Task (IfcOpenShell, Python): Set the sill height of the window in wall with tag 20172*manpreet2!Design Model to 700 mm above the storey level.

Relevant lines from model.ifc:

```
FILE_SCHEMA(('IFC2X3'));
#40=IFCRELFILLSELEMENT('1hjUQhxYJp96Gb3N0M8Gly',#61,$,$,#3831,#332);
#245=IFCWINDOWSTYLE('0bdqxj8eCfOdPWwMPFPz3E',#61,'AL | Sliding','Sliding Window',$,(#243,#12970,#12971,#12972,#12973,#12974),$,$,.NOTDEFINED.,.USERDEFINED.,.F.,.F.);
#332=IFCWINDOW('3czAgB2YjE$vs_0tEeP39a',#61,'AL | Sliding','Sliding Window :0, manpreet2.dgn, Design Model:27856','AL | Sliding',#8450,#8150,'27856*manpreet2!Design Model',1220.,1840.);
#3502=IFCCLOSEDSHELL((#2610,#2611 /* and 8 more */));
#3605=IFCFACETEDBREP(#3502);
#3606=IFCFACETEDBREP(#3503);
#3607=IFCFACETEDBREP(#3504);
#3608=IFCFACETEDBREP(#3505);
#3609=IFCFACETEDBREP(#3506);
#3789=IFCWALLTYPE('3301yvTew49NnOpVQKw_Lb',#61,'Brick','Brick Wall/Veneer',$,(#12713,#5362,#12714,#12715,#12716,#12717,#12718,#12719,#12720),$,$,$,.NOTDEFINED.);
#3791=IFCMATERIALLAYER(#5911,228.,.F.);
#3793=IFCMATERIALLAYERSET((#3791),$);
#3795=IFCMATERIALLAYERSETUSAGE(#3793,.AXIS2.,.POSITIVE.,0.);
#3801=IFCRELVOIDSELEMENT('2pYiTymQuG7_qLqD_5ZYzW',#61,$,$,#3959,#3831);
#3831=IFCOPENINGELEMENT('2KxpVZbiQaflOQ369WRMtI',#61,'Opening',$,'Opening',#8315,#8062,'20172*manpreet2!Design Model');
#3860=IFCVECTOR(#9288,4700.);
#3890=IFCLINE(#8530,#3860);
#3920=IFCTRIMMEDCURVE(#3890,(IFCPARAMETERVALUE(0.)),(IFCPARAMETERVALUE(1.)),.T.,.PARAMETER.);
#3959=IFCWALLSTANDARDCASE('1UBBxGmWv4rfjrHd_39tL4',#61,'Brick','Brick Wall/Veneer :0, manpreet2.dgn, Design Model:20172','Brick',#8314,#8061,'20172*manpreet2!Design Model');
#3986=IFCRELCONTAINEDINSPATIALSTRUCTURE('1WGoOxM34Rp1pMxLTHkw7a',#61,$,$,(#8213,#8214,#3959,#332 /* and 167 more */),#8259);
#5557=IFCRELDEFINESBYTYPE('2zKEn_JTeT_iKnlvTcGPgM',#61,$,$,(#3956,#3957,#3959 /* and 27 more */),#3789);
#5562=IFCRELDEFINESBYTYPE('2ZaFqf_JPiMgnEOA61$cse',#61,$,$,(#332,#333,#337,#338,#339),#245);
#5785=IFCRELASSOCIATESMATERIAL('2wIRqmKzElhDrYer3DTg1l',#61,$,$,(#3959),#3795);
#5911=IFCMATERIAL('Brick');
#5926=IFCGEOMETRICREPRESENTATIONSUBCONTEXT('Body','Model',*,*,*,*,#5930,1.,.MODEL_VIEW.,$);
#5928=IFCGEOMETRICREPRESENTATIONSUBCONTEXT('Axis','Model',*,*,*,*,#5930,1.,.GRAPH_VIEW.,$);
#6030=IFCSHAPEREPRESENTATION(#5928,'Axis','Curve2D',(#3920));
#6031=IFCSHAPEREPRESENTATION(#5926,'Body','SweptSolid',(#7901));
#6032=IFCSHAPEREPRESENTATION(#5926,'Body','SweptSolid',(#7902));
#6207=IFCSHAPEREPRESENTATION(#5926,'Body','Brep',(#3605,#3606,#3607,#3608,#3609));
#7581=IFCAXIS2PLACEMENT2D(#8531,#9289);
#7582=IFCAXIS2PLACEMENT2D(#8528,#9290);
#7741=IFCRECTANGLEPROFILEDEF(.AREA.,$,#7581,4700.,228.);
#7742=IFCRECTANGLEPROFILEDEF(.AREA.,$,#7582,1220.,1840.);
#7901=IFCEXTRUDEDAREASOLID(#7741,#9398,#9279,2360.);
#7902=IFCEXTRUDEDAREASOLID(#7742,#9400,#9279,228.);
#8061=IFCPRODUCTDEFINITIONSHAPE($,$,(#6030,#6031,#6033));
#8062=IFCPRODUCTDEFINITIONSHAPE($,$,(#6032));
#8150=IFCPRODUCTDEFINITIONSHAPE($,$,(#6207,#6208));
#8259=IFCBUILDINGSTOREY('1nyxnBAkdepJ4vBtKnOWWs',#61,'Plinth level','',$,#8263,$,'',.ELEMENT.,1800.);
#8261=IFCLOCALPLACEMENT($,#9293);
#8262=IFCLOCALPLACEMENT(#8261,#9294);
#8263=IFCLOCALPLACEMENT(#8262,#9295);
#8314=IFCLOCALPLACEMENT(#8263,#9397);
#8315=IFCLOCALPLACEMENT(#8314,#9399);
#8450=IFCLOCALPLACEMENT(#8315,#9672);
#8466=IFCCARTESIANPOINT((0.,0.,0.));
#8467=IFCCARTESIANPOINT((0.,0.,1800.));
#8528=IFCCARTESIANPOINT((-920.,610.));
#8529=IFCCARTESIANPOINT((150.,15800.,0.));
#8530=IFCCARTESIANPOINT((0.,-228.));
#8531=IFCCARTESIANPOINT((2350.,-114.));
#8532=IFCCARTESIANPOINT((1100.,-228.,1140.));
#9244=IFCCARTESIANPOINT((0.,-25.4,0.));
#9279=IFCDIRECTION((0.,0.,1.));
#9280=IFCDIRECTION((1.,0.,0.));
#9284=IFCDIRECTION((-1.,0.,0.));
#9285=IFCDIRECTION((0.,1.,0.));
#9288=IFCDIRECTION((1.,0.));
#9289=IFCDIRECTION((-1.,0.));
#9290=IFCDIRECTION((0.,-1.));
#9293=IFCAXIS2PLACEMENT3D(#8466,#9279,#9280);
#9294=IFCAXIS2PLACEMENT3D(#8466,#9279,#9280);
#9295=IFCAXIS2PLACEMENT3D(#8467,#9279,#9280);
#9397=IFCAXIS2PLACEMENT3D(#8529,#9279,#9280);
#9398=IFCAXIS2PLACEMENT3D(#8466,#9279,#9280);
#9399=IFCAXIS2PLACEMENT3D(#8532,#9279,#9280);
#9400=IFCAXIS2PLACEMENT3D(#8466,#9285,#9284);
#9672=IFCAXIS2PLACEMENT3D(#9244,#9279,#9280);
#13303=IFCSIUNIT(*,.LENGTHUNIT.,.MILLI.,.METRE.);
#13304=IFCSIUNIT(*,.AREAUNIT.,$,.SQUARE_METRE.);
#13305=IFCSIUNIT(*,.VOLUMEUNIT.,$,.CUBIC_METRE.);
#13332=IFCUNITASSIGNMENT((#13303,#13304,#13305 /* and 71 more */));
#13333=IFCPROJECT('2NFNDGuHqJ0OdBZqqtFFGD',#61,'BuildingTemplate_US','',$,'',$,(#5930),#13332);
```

```python
import numpy as np
import ifcopenshell
import ifcopenshell.api.geometry
import ifcopenshell.geom
import ifcopenshell.util.element
import ifcopenshell.util.placement
import ifcopenshell.util.shape
import ifcopenshell.util.unit

model = ifcopenshell.open("model.ifc")
unit_scale = ifcopenshell.util.unit.calculate_unit_scale(model)

window = model.by_guid("3czAgB2YjE$vs_0tEeP39a")
opening = window.FillsVoids[0].RelatingOpeningElement
storey = ifcopenshell.util.element.get_container(window, ifc_class="IfcBuildingStorey")
level = ifcopenshell.util.placement.get_local_placement(storey.ObjectPlacement)[2, 3]

# The opening's origin need not be at the sill, so measure its lowest point.
shape = ifcopenshell.geom.create_shape(ifcopenshell.geom.settings(), opening)
bottom = ifcopenshell.util.shape.get_shape_bottom_elevation(shape, shape.geometry) / unit_scale
dz = level + 0.7 / unit_scale - bottom

shift = np.array([0.0, 0.0, dz])
# The window is placed relative to its opening, so it follows when the opening moves.
matrix = ifcopenshell.util.placement.get_local_placement(opening.ObjectPlacement)
matrix[:3, 3] += shift
ifcopenshell.api.geometry.edit_object_placement(
    model, product=opening, matrix=matrix, is_si=False, should_transform_children=True
)

print(f"moved by {dz * unit_scale:+.3f} m")

model.write("model-out.ifc")
```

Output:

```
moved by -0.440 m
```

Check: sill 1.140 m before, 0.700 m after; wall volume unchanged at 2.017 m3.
